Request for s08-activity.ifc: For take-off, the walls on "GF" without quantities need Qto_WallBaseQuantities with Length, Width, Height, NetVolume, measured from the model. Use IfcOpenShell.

First a look at what the model holds.

```python
import ifcopenshell
import ifcopenshell.util.element
import ifcopenshell.util.unit

model = ifcopenshell.open("s08-activity.ifc")
print(model.schema)
for unit_type in ("LENGTHUNIT", "AREAUNIT", "VOLUMEUNIT"):
    print(unit_type, ifcopenshell.util.unit.calculate_unit_scale(model, unit_type))
storey = next(s for s in model.by_type("IfcBuildingStorey") if s.Name == "GF")
walls = [e for e in ifcopenshell.util.element.get_decomposition(storey) if e.is_a("IfcWall")]
for e in sorted(walls, key=lambda e: e.id()):
    print(e.id(), e.is_a(), e.Name, list(ifcopenshell.util.element.get_psets(e, qtos_only=True)), sep=" | ")
```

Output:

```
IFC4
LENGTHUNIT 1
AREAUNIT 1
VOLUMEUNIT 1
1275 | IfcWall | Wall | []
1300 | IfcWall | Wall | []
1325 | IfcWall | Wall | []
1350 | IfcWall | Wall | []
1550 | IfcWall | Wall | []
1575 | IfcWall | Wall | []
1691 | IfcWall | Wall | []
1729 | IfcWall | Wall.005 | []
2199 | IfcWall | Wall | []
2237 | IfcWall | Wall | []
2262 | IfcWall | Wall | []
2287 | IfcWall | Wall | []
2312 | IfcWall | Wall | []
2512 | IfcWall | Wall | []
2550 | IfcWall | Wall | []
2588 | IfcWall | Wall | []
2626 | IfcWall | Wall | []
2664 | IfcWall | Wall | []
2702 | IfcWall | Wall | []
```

```python
import ifcopenshell
import ifcopenshell.api.pset
import ifcopenshell.geom
import ifcopenshell.util.element
import ifcopenshell.util.shape
import ifcopenshell.util.unit

model = ifcopenshell.open("s08-activity.ifc")
unit_scale = ifcopenshell.util.unit.calculate_unit_scale(model)
volume_scale = ifcopenshell.util.unit.calculate_unit_scale(model, "VOLUMEUNIT")
settings = ifcopenshell.geom.settings()

storey = next(s for s in model.by_type("IfcBuildingStorey") if s.Name == "GF")
walls = [e for e in ifcopenshell.util.element.get_decomposition(storey) if e.is_a("IfcWall")]

for e in sorted(walls, key=lambda e: e.id()):
    if ifcopenshell.util.element.get_psets(e, qtos_only=True, should_inherit=False):
        continue
    # Geometry comes back in metres, in the element's own axes.
    shape = ifcopenshell.geom.create_shape(settings, e)
    values = {
        "Length": ifcopenshell.util.shape.get_x(shape.geometry) / unit_scale,
        "Width": ifcopenshell.util.shape.get_y(shape.geometry) / unit_scale,
        "Height": ifcopenshell.util.shape.get_z(shape.geometry) / unit_scale,
        "NetVolume": ifcopenshell.util.shape.get_volume(shape.geometry) / volume_scale,
    }
    qto = ifcopenshell.api.pset.add_qto(model, product=e, name="Qto_WallBaseQuantities")
    ifcopenshell.api.pset.edit_qto(model, qto=qto, properties=values)
    print(e.id(), {k: round(v, 3) for k, v in values.items()})

model.write("s08-activity-out.ifc")
```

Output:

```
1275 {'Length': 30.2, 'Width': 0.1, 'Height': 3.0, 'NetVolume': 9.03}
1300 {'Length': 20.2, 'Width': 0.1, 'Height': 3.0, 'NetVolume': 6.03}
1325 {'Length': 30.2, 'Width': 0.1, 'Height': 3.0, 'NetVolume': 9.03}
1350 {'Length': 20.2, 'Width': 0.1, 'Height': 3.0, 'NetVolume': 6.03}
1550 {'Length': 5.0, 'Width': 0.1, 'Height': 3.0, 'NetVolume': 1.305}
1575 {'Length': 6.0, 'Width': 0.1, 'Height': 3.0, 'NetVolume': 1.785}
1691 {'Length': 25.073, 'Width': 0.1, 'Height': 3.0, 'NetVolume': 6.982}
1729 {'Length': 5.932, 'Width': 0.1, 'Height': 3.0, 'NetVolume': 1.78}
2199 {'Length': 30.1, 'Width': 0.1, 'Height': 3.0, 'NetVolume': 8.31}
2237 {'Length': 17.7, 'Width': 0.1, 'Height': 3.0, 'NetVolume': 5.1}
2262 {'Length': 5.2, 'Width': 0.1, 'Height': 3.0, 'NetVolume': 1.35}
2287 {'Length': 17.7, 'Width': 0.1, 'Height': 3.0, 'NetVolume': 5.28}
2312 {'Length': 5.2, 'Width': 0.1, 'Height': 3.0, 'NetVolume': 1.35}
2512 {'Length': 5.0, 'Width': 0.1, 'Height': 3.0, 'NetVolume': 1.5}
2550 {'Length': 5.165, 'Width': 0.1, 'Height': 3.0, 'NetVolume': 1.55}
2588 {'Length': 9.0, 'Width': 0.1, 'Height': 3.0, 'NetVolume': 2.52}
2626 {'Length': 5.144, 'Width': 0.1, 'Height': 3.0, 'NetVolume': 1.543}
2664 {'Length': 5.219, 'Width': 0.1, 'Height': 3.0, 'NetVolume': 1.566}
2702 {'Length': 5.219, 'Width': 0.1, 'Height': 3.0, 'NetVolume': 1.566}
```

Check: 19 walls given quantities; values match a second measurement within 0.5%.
